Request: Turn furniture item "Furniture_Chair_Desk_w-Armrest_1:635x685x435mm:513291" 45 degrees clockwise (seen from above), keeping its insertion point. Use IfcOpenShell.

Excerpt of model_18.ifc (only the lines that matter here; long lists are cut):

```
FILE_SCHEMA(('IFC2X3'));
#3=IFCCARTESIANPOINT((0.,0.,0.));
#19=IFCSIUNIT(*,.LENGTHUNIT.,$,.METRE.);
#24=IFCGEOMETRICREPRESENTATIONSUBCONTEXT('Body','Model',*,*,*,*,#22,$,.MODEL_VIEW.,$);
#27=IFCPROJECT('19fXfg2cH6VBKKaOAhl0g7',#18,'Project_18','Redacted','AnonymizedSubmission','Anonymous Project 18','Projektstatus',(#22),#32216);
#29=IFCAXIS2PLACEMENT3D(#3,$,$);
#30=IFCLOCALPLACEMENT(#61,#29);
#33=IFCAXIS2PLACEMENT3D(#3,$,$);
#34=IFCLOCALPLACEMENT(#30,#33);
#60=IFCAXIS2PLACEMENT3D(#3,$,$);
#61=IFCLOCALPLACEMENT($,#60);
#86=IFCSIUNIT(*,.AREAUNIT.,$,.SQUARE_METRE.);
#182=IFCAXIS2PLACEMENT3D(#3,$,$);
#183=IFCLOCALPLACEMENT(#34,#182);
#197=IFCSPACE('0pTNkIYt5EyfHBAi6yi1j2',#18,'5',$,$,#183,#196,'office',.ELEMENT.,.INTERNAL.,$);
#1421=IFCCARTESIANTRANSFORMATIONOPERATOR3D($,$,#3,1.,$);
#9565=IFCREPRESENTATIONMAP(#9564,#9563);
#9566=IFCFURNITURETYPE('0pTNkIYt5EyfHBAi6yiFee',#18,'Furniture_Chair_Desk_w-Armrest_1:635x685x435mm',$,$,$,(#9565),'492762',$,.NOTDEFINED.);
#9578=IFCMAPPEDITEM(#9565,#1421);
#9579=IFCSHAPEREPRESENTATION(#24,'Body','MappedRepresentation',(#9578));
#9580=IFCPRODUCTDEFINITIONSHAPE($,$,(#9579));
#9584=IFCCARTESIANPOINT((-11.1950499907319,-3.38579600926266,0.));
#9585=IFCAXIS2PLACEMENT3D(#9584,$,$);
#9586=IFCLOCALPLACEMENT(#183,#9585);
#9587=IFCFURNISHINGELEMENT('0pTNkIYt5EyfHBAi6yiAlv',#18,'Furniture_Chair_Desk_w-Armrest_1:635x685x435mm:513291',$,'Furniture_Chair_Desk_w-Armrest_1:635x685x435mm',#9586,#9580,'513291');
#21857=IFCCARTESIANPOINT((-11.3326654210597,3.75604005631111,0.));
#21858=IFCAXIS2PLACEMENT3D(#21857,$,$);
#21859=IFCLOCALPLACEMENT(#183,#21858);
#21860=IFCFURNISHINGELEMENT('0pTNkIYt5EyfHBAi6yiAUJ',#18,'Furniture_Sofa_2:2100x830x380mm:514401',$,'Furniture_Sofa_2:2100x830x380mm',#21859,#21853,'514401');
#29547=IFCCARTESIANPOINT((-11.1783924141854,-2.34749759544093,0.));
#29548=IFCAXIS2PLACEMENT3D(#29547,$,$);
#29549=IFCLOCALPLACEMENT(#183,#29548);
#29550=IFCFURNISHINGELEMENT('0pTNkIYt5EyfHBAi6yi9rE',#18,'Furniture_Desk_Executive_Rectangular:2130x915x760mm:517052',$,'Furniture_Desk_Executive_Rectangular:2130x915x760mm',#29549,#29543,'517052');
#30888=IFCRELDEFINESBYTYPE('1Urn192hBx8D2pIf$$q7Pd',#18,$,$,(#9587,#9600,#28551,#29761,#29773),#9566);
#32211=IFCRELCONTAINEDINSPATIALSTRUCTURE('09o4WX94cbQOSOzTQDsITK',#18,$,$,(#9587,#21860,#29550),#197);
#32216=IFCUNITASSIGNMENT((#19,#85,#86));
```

```python
import ifcopenshell
import ifcopenshell.api.geometry
import ifcopenshell.util.placement

model = ifcopenshell.open("model_18.ifc")

item = model.by_guid("0pTNkIYt5EyfHBAi6yiAlv")
matrix = ifcopenshell.util.placement.get_local_placement(item.ObjectPlacement)
matrix = matrix @ ifcopenshell.util.placement.rotation(-45, "Z")
ifcopenshell.api.geometry.edit_object_placement(model, product=item, matrix=matrix, is_si=False)

print(ifcopenshell.util.placement.get_local_placement(item.ObjectPlacement).round(3) + 0.0)

model.write("model_18-out.ifc")
```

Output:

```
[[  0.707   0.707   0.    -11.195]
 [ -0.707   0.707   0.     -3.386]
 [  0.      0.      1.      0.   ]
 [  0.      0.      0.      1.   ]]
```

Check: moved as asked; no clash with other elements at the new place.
